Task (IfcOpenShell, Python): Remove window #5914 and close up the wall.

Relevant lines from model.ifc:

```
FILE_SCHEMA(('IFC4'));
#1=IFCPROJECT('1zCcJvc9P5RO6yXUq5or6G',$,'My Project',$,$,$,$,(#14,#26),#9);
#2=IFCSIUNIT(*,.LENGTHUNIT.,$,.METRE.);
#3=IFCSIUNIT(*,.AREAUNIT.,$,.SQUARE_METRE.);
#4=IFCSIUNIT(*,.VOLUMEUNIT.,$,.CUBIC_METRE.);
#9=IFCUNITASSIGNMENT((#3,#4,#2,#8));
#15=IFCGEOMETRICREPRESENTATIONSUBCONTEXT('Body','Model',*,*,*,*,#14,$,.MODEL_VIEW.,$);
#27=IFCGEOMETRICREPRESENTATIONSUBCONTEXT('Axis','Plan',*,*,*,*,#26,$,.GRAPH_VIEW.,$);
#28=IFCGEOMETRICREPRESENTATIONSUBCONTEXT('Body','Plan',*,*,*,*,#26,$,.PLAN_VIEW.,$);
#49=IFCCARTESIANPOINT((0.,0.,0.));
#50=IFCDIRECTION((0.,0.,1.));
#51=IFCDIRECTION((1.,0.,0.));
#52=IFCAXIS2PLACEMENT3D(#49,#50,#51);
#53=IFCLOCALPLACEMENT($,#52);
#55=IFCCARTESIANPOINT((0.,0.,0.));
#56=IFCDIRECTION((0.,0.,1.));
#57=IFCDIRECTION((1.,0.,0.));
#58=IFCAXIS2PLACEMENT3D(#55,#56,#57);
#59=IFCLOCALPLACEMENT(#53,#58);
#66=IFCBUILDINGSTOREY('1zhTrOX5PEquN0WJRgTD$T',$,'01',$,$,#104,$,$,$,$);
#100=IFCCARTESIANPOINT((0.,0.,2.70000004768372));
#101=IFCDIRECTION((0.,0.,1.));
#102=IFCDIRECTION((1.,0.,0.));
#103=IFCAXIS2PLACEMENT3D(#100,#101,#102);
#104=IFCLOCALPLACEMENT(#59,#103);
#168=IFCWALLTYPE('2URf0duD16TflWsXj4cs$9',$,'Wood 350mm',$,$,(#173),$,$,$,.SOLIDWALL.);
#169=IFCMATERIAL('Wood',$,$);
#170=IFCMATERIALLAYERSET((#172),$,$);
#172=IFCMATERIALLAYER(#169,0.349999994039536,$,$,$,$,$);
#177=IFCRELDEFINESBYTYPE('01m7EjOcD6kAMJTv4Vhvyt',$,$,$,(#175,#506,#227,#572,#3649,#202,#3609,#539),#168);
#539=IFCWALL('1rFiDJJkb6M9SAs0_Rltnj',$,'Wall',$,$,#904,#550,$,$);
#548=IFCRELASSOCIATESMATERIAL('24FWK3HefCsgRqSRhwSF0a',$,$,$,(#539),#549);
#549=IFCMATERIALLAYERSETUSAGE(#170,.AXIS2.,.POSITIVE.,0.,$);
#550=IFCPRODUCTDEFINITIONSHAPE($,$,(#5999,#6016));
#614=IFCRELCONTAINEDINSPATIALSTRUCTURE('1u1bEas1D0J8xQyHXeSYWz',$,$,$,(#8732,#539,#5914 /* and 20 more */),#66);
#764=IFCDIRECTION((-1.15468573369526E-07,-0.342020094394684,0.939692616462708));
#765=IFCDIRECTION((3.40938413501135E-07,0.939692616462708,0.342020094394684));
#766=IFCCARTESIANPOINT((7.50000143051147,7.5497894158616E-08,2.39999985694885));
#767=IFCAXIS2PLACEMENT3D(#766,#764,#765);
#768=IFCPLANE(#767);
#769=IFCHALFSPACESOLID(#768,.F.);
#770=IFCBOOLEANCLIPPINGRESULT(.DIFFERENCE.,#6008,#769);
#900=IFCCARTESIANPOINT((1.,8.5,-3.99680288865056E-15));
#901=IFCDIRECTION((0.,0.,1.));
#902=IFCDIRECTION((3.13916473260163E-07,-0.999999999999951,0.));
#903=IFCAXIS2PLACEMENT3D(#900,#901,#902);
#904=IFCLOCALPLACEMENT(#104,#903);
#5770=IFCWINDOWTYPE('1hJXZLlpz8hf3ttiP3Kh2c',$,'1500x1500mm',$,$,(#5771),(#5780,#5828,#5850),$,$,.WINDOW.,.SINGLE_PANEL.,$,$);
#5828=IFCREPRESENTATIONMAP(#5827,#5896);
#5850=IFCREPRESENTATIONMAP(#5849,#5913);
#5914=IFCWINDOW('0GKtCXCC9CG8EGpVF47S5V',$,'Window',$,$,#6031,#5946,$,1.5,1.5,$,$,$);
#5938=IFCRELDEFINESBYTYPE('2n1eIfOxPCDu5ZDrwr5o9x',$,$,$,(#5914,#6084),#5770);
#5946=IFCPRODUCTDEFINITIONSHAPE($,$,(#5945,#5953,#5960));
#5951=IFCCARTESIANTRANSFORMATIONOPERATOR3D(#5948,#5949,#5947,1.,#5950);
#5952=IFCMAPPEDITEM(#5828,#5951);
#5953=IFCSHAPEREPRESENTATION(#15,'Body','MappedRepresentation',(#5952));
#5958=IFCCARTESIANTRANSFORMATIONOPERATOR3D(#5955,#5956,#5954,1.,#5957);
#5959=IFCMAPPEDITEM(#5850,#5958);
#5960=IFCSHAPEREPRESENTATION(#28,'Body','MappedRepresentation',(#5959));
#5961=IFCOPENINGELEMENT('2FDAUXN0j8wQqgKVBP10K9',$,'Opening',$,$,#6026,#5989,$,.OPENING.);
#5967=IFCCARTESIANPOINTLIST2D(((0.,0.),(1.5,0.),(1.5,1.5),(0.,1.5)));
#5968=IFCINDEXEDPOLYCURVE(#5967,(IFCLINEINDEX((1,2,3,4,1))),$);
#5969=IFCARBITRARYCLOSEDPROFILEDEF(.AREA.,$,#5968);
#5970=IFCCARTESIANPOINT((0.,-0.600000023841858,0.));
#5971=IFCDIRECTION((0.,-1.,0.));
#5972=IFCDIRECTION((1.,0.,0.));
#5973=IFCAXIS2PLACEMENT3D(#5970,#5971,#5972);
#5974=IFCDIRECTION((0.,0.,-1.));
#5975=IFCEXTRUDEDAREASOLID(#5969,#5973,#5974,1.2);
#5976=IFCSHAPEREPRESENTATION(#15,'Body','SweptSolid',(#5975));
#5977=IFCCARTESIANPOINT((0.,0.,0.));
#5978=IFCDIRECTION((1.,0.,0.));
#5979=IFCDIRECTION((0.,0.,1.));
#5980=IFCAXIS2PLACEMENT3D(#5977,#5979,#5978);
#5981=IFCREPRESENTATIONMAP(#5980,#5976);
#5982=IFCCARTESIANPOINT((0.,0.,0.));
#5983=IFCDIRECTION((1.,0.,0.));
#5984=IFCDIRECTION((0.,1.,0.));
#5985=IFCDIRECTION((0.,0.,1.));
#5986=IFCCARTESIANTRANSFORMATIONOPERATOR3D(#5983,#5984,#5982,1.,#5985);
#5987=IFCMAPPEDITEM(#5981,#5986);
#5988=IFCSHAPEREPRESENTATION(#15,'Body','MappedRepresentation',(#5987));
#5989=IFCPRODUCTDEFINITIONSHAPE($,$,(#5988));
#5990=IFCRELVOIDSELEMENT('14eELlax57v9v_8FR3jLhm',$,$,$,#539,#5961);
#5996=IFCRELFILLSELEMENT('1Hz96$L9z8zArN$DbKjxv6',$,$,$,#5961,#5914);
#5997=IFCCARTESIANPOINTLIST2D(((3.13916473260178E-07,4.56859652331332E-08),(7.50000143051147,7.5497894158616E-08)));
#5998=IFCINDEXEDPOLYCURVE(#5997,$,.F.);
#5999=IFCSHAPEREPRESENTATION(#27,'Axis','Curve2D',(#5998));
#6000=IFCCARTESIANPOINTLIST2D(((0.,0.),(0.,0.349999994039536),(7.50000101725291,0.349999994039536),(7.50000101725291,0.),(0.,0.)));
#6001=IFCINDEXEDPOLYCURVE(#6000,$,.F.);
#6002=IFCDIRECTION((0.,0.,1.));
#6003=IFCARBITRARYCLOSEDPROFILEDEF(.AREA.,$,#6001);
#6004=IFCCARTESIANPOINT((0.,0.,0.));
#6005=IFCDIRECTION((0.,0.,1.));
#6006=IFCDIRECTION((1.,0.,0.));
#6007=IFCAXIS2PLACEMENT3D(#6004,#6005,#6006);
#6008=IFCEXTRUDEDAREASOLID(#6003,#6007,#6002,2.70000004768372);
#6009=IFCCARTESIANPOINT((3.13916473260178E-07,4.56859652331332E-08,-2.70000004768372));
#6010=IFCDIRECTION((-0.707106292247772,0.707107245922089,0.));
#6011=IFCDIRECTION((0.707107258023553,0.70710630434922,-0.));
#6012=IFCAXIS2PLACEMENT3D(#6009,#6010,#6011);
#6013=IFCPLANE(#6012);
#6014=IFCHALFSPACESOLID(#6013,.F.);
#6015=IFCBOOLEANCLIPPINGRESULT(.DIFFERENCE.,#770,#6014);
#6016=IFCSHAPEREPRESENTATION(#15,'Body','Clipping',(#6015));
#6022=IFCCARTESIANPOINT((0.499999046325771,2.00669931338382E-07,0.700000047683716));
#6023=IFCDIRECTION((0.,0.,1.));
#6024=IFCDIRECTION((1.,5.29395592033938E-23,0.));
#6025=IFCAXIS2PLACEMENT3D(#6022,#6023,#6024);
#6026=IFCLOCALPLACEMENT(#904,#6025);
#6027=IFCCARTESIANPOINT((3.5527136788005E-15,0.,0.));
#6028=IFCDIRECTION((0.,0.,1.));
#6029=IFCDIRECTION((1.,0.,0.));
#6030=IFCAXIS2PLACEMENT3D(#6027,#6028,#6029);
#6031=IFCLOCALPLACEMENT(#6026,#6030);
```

```python
import ifcopenshell
import ifcopenshell.api.feature
import ifcopenshell.api.root
import ifcopenshell.geom
import ifcopenshell.util.shape

model = ifcopenshell.open("model.ifc")
settings = ifcopenshell.geom.settings()


def volume(element):
    """Net volume in cubic metres, openings subtracted."""
    shape = ifcopenshell.geom.create_shape(settings, element)
    return ifcopenshell.util.shape.get_volume(shape.geometry)


window = model.by_guid("0GKtCXCC9CG8EGpVF47S5V")
opening = window.FillsVoids[0].RelatingOpeningElement
wall = opening.VoidsElements[0].RelatingBuildingElement
before = volume(wall)

ifcopenshell.api.root.remove_product(model, product=window)
ifcopenshell.api.feature.remove_feature(model, feature=opening)

after = volume(wall)

print(f"wall volume {before:.3f} -> {after:.3f} m3")

model.write("model_rev.ifc")
```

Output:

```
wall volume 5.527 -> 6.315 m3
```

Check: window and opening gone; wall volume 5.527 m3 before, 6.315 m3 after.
